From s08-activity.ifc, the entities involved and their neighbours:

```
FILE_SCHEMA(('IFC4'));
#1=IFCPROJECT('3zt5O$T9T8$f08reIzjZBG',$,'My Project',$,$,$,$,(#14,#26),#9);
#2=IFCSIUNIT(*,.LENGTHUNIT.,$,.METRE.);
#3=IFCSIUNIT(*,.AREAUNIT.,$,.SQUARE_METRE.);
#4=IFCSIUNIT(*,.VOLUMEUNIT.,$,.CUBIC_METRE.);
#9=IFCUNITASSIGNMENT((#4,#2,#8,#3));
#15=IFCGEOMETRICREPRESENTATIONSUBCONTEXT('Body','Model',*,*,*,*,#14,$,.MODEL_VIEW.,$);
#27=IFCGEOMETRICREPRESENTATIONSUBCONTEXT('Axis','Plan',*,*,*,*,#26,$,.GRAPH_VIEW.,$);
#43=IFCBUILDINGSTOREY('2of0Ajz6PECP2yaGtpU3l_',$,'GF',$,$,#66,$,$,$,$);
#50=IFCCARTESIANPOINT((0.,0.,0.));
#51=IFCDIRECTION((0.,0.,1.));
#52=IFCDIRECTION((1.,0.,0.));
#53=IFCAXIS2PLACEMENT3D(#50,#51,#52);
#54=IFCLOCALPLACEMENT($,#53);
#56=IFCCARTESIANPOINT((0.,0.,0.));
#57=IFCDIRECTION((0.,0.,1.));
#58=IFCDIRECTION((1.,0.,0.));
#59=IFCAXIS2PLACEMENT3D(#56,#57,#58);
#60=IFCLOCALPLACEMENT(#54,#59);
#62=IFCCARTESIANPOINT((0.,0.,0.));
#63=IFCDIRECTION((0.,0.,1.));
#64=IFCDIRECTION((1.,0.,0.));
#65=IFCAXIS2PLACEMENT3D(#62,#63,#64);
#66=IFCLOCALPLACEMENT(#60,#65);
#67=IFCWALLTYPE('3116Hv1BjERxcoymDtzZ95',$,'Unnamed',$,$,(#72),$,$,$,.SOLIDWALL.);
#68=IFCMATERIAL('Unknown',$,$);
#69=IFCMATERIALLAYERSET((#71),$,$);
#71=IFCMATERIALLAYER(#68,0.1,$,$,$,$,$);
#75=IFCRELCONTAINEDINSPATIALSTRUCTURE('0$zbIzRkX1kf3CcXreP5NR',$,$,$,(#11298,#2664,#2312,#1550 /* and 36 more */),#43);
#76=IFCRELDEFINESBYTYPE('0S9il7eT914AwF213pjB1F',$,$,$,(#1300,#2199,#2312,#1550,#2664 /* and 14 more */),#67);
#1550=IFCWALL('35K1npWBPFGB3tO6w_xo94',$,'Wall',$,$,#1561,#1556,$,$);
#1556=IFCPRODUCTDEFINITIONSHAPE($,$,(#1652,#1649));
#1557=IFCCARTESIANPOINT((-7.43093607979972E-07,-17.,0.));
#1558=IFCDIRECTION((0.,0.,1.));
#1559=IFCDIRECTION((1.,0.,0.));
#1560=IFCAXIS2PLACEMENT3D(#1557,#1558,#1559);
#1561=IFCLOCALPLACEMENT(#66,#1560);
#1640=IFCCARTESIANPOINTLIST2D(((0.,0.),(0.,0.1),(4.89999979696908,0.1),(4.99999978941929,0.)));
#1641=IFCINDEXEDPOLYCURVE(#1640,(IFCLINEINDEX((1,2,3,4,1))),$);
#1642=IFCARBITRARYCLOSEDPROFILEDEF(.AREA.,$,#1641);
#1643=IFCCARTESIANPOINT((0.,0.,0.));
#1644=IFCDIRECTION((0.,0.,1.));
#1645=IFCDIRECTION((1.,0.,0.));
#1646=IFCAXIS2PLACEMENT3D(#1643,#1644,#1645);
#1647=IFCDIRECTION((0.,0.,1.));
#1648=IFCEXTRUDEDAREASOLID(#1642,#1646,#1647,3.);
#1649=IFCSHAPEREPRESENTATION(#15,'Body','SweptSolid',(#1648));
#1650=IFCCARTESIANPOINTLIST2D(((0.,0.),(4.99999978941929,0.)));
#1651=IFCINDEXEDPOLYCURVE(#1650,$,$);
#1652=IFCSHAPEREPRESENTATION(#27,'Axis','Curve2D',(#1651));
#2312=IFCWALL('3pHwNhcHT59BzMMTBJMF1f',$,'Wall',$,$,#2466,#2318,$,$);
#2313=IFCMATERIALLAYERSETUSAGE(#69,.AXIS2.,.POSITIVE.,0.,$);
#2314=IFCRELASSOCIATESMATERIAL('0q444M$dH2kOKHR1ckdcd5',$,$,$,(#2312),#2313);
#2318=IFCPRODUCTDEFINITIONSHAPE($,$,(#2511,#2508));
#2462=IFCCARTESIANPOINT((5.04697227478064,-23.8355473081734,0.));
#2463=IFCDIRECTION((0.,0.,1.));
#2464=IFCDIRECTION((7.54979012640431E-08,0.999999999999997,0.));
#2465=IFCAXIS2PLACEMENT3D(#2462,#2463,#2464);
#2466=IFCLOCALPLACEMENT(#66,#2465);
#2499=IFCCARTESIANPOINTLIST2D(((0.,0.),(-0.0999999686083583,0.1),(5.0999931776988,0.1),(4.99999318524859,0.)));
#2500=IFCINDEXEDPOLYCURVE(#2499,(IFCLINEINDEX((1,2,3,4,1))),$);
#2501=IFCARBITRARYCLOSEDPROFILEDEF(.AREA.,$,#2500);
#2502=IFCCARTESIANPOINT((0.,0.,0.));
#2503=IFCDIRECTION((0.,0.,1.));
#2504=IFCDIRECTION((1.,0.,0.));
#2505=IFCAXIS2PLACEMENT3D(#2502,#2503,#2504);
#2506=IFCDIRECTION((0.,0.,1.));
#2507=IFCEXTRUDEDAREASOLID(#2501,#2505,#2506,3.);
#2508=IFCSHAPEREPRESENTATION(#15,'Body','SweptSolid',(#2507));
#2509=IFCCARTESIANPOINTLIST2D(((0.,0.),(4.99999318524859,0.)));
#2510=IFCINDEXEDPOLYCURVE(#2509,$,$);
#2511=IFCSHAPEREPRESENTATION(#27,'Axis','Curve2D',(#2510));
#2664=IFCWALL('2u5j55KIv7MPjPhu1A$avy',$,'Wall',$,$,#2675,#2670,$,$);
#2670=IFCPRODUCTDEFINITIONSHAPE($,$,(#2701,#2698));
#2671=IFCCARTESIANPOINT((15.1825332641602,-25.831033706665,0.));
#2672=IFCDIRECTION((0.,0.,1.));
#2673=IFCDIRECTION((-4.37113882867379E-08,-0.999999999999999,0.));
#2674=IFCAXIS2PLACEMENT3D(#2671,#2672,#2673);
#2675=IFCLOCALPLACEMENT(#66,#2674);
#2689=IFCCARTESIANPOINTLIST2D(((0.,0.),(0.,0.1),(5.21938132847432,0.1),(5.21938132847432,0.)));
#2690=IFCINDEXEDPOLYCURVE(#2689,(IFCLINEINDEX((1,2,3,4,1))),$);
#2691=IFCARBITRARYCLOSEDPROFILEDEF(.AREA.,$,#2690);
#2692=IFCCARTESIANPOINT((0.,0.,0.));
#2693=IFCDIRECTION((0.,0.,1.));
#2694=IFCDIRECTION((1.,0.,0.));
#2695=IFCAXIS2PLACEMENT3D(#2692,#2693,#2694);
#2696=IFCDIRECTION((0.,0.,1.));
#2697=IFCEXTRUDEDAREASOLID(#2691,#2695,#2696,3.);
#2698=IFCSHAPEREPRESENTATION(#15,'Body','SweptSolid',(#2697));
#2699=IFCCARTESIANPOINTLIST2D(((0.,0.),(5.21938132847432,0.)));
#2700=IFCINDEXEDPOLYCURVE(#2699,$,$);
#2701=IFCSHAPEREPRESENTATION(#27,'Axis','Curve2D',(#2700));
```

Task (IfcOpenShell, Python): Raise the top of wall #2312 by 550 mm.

```python
import ifcopenshell
import ifcopenshell.geom
import ifcopenshell.util.representation
import ifcopenshell.util.shape

model = ifcopenshell.open("s08-activity.ifc")
settings = ifcopenshell.geom.settings()


def volume(element):
    """Net volume in cubic metres, openings subtracted."""
    shape = ifcopenshell.geom.create_shape(settings, element)
    return ifcopenshell.util.shape.get_volume(shape.geometry)


wall = model.by_guid("3pHwNhcHT59BzMMTBJMF1f")
before = volume(wall)

body = ifcopenshell.util.representation.get_representation(wall, "Model", "Body")
solid = body.Items[0]
old_height = solid.Depth
solid.Depth += 0.55
after = volume(wall)

print(f"height {old_height:g} -> {solid.Depth:g}, volume {before:.3f} -> {after:.3f} m3")

model.write("s08-activity_updated.ifc")
```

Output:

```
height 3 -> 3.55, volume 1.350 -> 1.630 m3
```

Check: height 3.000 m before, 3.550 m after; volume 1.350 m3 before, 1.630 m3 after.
